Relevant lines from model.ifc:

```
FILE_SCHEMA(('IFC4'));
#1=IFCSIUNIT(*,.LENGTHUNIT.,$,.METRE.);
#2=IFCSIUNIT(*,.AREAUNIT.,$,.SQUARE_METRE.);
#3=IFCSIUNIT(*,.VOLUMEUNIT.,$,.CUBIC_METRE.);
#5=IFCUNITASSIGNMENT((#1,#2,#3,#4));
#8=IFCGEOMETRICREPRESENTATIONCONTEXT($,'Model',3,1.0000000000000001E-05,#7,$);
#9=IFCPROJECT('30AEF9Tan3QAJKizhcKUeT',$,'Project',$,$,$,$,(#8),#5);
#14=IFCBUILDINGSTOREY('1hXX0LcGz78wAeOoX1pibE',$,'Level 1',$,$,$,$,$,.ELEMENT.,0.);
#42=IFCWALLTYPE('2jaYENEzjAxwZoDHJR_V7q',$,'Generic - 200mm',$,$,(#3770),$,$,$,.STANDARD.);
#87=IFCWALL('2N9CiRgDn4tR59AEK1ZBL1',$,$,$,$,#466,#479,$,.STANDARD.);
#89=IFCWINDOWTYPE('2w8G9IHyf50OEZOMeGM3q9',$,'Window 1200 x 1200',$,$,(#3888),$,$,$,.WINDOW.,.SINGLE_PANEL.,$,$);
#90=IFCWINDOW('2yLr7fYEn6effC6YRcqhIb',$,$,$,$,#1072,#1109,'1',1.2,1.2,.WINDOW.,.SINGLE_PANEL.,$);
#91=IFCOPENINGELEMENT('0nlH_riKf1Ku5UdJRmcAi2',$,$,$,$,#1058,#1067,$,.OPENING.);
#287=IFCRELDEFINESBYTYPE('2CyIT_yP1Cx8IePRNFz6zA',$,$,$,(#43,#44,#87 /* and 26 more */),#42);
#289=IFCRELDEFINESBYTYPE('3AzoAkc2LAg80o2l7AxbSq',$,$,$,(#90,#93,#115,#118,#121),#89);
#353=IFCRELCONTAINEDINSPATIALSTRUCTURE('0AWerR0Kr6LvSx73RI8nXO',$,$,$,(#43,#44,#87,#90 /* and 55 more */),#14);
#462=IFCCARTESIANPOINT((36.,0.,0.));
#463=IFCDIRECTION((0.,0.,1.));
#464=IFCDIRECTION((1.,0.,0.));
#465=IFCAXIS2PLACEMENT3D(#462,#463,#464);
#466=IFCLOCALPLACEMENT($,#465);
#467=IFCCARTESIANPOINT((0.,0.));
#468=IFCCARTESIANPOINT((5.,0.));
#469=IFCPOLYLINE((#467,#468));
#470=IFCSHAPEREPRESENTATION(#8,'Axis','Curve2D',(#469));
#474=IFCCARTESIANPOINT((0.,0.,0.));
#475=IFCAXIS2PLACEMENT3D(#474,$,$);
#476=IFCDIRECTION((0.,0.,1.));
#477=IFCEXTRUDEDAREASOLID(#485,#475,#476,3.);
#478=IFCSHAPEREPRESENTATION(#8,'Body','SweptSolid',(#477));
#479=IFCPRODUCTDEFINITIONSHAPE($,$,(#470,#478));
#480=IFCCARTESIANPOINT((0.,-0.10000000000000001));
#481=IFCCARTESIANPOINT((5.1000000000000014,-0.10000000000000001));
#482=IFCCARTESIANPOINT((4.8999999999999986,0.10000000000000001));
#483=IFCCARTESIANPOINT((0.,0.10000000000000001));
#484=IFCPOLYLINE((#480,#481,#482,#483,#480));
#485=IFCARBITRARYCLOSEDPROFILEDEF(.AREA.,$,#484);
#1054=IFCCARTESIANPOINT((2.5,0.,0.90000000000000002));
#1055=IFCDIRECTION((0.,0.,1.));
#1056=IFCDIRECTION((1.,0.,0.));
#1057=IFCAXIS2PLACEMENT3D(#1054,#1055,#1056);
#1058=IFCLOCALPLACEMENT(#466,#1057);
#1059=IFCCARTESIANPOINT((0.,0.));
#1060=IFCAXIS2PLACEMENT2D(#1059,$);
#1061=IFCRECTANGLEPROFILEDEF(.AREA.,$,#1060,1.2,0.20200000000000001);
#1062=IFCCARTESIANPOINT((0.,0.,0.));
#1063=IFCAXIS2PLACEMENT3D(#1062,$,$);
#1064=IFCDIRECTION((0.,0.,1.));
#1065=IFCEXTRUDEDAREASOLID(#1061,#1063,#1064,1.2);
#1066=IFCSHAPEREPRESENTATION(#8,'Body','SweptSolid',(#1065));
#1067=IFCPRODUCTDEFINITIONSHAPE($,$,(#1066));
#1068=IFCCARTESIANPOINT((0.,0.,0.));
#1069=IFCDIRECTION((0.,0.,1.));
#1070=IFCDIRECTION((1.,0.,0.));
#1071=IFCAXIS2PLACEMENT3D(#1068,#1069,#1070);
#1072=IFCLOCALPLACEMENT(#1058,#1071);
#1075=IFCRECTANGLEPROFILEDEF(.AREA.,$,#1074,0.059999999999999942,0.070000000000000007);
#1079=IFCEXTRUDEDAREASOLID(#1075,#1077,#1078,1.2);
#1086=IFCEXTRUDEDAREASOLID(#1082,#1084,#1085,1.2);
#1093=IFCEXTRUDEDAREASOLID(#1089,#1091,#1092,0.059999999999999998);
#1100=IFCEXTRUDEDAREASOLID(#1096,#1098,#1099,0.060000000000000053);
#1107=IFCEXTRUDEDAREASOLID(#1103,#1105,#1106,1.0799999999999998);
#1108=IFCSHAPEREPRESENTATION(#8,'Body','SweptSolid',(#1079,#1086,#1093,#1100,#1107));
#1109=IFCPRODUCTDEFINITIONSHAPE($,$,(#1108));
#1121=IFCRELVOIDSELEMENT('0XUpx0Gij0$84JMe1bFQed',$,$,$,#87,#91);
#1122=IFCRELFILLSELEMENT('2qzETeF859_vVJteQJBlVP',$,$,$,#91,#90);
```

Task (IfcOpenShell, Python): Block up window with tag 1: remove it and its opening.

```python
import ifcopenshell
import ifcopenshell.api.feature
import ifcopenshell.api.root
import ifcopenshell.geom
import ifcopenshell.util.shape

model = ifcopenshell.open("model.ifc")
settings = ifcopenshell.geom.settings()


def volume(element):
    """Net volume in cubic metres, openings subtracted."""
    shape = ifcopenshell.geom.create_shape(settings, element)
    return ifcopenshell.util.shape.get_volume(shape.geometry)


window = model.by_id(90)
opening = window.FillsVoids[0].RelatingOpeningElement
wall = opening.VoidsElements[0].RelatingBuildingElement
before = volume(wall)

ifcopenshell.api.root.remove_product(model, product=window)
ifcopenshell.api.feature.remove_feature(model, feature=opening)

after = volume(wall)

print(f"wall volume {before:.3f} -> {after:.3f} m3")

model.write("model_updated.ifc")
```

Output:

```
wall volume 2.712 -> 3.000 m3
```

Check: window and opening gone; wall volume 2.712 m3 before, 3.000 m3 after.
